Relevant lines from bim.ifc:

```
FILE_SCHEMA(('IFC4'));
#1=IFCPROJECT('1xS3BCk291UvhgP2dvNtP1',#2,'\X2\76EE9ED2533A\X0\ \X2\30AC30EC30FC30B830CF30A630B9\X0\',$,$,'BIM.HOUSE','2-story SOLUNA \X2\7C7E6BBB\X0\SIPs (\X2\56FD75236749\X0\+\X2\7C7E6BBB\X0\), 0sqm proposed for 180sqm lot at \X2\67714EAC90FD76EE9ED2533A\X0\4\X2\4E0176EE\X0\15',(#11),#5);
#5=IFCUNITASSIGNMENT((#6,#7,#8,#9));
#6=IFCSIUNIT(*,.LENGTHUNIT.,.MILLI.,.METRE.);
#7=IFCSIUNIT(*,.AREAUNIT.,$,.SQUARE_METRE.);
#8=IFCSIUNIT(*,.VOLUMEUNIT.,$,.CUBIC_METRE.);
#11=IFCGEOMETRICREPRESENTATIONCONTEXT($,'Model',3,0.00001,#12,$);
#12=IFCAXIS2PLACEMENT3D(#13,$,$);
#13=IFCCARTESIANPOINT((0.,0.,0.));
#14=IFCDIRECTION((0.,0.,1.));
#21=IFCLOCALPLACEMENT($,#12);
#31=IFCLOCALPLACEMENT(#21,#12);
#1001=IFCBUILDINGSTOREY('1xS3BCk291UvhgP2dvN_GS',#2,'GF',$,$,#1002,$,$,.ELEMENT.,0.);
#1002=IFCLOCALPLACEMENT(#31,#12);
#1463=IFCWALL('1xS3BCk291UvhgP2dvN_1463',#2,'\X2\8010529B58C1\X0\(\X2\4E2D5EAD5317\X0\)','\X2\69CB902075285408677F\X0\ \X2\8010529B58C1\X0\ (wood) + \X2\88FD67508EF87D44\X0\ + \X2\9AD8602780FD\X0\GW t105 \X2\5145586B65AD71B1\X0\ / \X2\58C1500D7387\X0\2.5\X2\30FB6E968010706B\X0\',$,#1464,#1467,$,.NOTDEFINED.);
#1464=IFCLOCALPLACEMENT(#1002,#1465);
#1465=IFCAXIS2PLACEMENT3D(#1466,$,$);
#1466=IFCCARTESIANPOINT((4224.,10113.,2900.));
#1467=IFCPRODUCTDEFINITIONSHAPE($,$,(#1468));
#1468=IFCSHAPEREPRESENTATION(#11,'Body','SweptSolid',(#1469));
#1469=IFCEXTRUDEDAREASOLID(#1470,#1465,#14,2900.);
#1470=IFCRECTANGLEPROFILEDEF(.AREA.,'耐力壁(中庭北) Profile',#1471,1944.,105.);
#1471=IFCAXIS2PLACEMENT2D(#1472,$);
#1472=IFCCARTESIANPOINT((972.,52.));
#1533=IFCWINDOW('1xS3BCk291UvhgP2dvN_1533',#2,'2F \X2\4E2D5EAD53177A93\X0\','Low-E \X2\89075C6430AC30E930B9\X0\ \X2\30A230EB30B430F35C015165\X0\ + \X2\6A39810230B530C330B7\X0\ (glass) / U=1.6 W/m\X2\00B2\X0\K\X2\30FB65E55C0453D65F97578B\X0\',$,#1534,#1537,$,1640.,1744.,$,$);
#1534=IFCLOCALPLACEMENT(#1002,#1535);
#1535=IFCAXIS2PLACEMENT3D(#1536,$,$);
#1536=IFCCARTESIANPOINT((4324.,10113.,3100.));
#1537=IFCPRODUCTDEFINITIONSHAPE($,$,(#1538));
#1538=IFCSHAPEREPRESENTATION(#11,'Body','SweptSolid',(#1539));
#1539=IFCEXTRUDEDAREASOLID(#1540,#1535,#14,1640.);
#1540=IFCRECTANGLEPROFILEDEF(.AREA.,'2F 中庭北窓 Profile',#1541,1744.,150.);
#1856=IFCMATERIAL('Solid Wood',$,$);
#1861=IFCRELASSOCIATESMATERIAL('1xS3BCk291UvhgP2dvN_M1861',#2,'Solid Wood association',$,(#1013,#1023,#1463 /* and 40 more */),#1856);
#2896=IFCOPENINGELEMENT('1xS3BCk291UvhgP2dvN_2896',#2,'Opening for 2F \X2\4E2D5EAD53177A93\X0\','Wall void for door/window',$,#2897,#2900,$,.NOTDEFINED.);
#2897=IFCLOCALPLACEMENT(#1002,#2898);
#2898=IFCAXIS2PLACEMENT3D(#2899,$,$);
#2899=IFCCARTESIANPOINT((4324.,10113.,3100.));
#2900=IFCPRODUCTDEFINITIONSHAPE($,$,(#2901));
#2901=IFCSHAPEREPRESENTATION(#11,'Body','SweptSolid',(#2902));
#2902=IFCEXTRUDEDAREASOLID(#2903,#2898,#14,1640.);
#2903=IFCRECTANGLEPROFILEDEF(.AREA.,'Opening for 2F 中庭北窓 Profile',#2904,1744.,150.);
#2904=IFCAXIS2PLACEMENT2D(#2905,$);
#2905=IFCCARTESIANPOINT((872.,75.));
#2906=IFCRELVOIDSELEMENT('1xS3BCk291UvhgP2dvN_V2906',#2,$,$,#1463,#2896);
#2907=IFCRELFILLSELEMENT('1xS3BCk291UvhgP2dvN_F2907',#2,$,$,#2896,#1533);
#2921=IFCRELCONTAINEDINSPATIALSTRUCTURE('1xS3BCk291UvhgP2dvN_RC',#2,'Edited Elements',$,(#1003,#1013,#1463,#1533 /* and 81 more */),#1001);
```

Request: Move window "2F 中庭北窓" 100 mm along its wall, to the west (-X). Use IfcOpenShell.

```python
import ifcopenshell
import ifcopenshell.api.geometry
import ifcopenshell.util.placement

model = ifcopenshell.open("bim.ifc")

window = model.by_guid("1xS3BCk291UvhgP2dvN_1533")
opening = window.FillsVoids[0].RelatingOpeningElement
wall = opening.VoidsElements[0].RelatingBuildingElement

wall_matrix = ifcopenshell.util.placement.get_local_placement(wall.ObjectPlacement)
shift = wall_matrix[:3, 0] * -100.0
before = ifcopenshell.util.placement.get_local_placement(window.ObjectPlacement)[:3, 3].copy()

# The window is not placed relative to its opening, so move both.
for product in (opening, window):
    matrix = ifcopenshell.util.placement.get_local_placement(product.ObjectPlacement)
    matrix[:3, 3] += shift
    ifcopenshell.api.geometry.edit_object_placement(model, product=product, matrix=matrix, is_si=False)

after = ifcopenshell.util.placement.get_local_placement(window.ObjectPlacement)[:3, 3]
print("window moved by", (after - before).round(3) + 0.0)

model.write("bim_v2.ifc")
```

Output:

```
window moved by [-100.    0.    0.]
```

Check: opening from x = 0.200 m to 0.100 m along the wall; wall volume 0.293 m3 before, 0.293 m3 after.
